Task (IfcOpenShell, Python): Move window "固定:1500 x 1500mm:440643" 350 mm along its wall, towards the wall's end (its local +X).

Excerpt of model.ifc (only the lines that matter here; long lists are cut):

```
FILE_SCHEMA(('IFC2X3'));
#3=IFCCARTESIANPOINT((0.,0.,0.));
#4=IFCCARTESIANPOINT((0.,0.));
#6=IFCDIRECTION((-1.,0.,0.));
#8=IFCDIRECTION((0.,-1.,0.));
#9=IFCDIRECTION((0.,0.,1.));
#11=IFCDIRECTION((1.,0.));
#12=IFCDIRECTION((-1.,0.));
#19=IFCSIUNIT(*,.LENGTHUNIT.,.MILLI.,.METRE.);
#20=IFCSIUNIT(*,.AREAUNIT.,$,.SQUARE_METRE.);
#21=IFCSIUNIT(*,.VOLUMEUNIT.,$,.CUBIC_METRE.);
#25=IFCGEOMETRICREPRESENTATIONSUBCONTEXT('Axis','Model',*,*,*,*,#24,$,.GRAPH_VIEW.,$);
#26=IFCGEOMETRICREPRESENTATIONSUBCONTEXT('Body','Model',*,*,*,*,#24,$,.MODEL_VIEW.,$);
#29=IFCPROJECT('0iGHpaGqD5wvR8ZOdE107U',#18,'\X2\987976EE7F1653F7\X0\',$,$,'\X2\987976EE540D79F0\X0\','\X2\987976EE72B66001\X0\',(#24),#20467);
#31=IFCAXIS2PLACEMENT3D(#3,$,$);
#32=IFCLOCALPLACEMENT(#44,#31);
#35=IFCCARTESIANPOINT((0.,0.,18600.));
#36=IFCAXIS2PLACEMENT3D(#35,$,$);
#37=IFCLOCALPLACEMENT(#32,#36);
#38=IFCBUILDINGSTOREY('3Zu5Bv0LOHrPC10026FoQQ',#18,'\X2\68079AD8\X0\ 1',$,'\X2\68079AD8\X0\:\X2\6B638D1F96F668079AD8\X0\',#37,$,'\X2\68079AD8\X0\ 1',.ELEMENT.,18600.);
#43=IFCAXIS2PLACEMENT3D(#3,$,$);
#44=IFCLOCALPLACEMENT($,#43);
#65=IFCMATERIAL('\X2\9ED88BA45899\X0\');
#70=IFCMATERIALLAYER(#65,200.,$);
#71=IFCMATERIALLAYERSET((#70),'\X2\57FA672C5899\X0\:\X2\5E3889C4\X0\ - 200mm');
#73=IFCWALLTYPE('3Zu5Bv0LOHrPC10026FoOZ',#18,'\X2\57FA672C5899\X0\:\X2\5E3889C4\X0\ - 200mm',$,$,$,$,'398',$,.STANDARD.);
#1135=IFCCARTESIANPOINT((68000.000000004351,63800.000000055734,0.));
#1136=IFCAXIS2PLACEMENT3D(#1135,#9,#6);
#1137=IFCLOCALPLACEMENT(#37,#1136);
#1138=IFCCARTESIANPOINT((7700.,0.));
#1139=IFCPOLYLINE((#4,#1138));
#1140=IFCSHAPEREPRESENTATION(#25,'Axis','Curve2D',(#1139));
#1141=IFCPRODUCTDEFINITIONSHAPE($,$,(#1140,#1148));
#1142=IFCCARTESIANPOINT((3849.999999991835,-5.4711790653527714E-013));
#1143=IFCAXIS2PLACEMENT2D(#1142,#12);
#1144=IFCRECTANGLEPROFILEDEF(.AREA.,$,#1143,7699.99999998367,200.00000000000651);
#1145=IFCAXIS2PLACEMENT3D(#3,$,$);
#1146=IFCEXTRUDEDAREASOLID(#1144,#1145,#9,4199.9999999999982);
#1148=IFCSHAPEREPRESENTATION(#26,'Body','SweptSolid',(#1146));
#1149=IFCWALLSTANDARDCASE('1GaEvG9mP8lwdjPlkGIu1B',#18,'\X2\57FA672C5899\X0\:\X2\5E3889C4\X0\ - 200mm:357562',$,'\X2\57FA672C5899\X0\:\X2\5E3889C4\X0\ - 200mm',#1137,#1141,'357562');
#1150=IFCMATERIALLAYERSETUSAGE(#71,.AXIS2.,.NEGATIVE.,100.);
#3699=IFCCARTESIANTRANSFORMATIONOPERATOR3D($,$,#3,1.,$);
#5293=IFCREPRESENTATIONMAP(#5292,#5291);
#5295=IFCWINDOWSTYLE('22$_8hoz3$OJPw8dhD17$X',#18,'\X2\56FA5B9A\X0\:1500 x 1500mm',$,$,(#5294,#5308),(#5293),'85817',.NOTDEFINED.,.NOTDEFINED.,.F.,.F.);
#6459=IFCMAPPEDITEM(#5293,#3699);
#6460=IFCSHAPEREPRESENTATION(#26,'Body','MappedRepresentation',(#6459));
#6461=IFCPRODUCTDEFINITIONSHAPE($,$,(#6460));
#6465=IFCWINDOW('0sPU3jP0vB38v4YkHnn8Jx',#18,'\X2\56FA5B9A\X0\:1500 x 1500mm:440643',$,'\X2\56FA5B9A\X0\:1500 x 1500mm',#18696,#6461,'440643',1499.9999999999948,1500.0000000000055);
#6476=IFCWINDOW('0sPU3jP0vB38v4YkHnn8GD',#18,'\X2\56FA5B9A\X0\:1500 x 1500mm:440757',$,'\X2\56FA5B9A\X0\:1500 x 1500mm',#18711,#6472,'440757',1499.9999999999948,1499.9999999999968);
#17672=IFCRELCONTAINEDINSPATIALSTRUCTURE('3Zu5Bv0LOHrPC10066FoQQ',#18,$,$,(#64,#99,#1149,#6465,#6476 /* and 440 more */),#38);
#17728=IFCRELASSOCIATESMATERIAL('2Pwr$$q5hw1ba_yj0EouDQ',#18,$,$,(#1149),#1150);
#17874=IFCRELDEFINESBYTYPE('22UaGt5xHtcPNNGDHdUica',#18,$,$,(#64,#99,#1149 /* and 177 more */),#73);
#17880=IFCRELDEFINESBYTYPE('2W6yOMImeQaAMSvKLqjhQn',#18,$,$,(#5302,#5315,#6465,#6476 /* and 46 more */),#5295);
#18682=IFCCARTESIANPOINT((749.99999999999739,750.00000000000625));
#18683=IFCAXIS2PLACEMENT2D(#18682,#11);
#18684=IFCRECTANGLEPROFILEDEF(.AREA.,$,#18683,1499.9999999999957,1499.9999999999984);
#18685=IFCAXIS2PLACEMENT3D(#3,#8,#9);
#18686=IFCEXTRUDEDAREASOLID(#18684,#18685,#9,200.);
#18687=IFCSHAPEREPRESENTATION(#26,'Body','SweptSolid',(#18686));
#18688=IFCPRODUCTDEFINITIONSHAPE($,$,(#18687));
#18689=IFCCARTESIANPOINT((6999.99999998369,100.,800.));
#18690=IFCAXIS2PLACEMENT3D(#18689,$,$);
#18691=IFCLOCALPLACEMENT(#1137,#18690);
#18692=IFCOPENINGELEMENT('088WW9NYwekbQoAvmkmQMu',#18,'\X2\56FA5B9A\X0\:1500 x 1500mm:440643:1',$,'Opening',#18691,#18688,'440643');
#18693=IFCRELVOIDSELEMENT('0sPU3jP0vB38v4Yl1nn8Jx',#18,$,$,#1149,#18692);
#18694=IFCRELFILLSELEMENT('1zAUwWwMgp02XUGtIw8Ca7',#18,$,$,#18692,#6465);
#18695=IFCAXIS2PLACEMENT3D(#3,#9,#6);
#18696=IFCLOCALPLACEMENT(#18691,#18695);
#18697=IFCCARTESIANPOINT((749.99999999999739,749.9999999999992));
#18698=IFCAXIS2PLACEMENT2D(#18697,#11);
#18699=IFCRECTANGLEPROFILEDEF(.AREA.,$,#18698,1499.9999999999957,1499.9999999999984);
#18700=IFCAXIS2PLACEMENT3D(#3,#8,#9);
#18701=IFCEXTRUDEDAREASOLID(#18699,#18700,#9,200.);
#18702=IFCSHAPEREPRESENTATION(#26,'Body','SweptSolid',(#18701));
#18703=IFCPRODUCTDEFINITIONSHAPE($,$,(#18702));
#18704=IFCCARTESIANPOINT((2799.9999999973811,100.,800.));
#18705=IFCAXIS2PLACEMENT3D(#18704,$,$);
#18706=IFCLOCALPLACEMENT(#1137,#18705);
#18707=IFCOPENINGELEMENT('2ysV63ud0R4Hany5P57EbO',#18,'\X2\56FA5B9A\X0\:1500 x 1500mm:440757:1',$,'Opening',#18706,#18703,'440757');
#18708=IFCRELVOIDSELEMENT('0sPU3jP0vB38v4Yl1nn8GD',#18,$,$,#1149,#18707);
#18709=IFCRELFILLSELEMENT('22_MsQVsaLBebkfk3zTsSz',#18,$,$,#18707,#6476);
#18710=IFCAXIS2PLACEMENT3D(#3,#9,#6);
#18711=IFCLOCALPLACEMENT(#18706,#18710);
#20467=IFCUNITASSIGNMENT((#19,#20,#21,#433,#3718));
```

```python
import ifcopenshell
import ifcopenshell.api.geometry
import ifcopenshell.util.placement
import ifcopenshell.util.unit

model = ifcopenshell.open("model.ifc")
unit_scale = ifcopenshell.util.unit.calculate_unit_scale(model)

window = model.by_guid("0sPU3jP0vB38v4YkHnn8Jx")
opening = window.FillsVoids[0].RelatingOpeningElement
wall = opening.VoidsElements[0].RelatingBuildingElement

wall_matrix = ifcopenshell.util.placement.get_local_placement(wall.ObjectPlacement)
shift = wall_matrix[:3, 0] * 0.35 / unit_scale
before = ifcopenshell.util.placement.get_local_placement(window.ObjectPlacement)[:3, 3].copy()

# The window is placed relative to its opening, so it follows when the opening moves.
matrix = ifcopenshell.util.placement.get_local_placement(opening.ObjectPlacement)
matrix[:3, 3] += shift
ifcopenshell.api.geometry.edit_object_placement(
    model, product=opening, matrix=matrix, is_si=False, should_transform_children=True
)

after = ifcopenshell.util.placement.get_local_placement(window.ObjectPlacement)[:3, 3]
print("window moved by", (after - before).round(3) + 0.0)

model.write("model_updated.ifc")
```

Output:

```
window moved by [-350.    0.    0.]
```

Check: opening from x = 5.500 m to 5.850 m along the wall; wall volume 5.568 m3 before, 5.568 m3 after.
